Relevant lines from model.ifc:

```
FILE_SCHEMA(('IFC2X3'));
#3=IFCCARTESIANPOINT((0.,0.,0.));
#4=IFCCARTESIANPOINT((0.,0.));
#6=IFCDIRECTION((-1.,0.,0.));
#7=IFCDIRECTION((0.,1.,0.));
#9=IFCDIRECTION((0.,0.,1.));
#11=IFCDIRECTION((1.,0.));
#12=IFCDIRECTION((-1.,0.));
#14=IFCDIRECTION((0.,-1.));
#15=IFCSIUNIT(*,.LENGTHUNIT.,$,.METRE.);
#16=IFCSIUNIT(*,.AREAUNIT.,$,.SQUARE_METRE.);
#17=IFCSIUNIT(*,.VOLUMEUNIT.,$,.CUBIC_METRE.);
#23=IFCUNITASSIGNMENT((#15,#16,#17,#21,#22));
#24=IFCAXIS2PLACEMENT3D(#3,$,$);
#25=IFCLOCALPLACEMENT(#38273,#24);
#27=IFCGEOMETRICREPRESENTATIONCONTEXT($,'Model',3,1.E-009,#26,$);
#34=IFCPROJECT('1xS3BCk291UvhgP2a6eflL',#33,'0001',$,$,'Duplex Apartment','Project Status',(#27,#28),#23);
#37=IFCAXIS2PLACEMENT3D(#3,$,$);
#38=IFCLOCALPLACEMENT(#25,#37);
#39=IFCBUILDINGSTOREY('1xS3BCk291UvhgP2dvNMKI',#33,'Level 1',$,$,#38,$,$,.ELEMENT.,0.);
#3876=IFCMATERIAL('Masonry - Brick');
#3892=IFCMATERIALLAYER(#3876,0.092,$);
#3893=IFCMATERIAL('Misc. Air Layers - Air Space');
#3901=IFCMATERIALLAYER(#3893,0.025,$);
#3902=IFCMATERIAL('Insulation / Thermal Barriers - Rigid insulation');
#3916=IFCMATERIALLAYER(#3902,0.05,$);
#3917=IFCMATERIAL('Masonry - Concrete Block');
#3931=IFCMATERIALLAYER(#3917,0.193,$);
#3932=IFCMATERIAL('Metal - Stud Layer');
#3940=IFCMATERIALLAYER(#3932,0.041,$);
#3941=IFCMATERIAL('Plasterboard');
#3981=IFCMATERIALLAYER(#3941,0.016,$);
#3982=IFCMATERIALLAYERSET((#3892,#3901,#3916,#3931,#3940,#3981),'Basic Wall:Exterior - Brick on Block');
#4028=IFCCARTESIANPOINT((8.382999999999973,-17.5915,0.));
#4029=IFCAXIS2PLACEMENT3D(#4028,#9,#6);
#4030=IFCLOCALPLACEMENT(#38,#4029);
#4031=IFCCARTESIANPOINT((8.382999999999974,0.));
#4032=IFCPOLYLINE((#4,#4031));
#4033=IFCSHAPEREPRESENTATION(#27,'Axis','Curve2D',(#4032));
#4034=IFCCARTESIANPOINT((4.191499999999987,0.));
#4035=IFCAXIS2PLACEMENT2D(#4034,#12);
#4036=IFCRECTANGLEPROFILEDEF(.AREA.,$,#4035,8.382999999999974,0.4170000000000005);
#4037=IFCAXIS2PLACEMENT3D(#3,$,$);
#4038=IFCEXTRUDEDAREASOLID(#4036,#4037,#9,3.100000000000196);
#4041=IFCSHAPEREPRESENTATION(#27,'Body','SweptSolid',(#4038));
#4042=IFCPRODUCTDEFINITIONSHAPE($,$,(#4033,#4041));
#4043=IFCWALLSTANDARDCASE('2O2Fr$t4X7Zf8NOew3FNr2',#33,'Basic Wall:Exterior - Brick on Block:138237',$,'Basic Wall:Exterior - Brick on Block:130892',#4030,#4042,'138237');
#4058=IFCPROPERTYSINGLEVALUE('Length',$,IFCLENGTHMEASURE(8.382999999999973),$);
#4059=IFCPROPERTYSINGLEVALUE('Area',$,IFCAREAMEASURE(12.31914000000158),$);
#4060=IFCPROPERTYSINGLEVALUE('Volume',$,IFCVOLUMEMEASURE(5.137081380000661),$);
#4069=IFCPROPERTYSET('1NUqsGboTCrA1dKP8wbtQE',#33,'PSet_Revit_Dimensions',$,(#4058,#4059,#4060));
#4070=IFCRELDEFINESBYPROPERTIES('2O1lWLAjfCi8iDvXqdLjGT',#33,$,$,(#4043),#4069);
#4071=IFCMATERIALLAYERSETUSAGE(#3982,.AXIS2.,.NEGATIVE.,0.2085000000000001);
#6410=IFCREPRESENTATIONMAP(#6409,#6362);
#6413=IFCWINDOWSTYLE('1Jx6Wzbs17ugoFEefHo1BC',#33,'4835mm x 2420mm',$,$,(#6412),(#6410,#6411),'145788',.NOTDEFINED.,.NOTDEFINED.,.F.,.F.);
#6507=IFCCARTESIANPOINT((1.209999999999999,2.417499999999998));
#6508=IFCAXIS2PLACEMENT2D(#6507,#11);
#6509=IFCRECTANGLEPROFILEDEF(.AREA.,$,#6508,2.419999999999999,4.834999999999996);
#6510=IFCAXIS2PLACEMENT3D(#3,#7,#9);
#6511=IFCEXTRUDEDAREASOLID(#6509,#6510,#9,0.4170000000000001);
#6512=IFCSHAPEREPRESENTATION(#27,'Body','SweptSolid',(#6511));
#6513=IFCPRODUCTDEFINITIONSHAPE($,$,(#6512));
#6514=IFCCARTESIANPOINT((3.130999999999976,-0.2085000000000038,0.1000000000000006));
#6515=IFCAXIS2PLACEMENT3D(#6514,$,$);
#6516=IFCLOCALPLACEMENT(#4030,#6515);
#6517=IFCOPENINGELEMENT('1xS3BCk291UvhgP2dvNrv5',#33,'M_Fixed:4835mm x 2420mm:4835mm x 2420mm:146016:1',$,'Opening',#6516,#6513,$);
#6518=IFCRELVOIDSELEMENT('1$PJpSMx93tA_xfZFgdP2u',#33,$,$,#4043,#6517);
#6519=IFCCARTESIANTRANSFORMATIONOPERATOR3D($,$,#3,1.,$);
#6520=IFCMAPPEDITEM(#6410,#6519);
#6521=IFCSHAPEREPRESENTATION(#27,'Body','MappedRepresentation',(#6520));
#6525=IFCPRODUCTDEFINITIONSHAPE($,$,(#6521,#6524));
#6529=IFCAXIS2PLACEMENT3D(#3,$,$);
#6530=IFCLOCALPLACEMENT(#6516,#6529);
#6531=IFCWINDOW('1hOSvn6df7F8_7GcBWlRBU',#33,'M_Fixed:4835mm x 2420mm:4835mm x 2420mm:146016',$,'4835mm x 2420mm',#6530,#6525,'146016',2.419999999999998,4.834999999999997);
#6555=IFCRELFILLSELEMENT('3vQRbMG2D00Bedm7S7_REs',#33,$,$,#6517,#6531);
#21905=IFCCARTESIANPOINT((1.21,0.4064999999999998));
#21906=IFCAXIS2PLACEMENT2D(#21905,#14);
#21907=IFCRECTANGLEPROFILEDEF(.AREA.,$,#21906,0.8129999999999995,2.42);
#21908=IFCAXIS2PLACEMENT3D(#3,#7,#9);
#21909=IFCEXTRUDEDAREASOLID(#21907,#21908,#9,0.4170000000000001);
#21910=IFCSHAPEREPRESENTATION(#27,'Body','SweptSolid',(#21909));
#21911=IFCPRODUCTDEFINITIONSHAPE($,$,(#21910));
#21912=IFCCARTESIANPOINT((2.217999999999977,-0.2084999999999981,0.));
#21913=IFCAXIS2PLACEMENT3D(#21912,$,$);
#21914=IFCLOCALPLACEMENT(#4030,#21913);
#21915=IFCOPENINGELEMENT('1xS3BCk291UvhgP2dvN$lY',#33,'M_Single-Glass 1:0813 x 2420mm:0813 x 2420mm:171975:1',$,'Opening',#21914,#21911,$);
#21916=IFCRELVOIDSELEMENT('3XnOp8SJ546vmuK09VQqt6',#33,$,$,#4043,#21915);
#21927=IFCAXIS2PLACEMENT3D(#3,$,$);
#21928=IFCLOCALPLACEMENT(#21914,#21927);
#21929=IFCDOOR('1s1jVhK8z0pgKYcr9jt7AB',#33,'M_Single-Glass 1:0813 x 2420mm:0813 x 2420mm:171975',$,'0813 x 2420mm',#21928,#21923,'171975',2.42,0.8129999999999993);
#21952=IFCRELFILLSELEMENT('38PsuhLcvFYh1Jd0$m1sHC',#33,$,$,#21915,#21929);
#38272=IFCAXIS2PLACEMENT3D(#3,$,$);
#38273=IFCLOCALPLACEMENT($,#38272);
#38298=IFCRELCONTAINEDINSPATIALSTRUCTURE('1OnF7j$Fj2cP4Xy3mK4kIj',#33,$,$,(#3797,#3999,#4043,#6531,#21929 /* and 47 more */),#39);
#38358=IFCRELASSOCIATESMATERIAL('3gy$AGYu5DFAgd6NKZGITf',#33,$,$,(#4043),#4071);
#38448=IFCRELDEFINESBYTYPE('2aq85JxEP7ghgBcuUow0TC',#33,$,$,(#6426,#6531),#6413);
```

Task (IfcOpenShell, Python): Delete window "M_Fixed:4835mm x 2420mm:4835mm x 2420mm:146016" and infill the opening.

```python
import ifcopenshell
import ifcopenshell.api.feature
import ifcopenshell.api.pset
import ifcopenshell.api.root
import ifcopenshell.geom
import ifcopenshell.util.element
import ifcopenshell.util.shape
import ifcopenshell.util.unit

model = ifcopenshell.open("model.ifc")
area_scale = ifcopenshell.util.unit.calculate_unit_scale(model, "AREAUNIT")
volume_scale = ifcopenshell.util.unit.calculate_unit_scale(model, "VOLUMEUNIT")
settings = ifcopenshell.geom.settings()


def volume(element):
    """Net volume in cubic metres, openings subtracted."""
    shape = ifcopenshell.geom.create_shape(settings, element)
    return ifcopenshell.util.shape.get_volume(shape.geometry)


window = model.by_id(6531)
opening = window.FillsVoids[0].RelatingOpeningElement
wall = opening.VoidsElements[0].RelatingBuildingElement
before = volume(wall)

ifcopenshell.api.root.remove_product(model, product=window)
ifcopenshell.api.feature.remove_feature(model, feature=opening)

after = volume(wall)
thickness = 0.417  # wall thickness in metres

# Update the wall's stored quantities.
pset = model.by_id(ifcopenshell.util.element.get_pset(wall, "PSet_Revit_Dimensions", should_inherit=False)["id"])
ifcopenshell.api.pset.edit_pset(model, pset=pset, properties={
    "Area": model.create_entity("IfcAreaMeasure", after / thickness / area_scale),
    "Volume": model.create_entity("IfcVolumeMeasure", after / volume_scale),
})

print(f"wall volume {before:.3f} -> {after:.3f} m3")

model.write("model-out.ifc")
```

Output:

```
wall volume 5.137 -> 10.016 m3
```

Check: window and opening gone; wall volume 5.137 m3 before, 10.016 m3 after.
